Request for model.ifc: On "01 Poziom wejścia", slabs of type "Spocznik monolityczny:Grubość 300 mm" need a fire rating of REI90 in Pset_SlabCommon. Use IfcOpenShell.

First a look at what the model holds.

```python
import ifcopenshell
import ifcopenshell.util.element

model = ifcopenshell.open("model.ifc")
print(model.schema)
storey = next(s for s in model.by_type("IfcBuildingStorey") if s.Name == "01 Poziom wejścia")
slabs = [e for e in ifcopenshell.util.element.get_decomposition(storey) if e.is_a("IfcSlab")]
seen = {}
for e in slabs:
    element_type = ifcopenshell.util.element.get_type(e)
    key = (element_type.Name if element_type != e and element_type else None, ifcopenshell.util.element.get_pset(e, "Pset_SlabCommon", "FireRating"))
    seen[key] = seen.get(key, 0) + 1
for (name, value), count in sorted(seen.items(), key=str):
    print(count, "x", name, "|", value)
```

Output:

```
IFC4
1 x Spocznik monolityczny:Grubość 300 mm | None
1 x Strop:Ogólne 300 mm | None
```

```python
import ifcopenshell
import ifcopenshell.api.pset
import ifcopenshell.util.element

model = ifcopenshell.open("model.ifc")

storey = next(s for s in model.by_type("IfcBuildingStorey") if s.Name == "01 Poziom wejścia")
slabs = [e for e in ifcopenshell.util.element.get_decomposition(storey) if e.is_a("IfcSlab")]

count = 0
for e in slabs:
    element_type = ifcopenshell.util.element.get_type(e)
    if element_type in (None, e) or element_type.Name != "Spocznik monolityczny:Grubość 300 mm":
        continue
    # add_pset returns the element's existing set when there is one.
    pset = ifcopenshell.api.pset.add_pset(model, product=e, name="Pset_SlabCommon")
    ifcopenshell.api.pset.edit_pset(model, pset=pset, properties={"FireRating": "REI90"})
    count += 1

print(count, "slabs updated")

model.write("model_updated.ifc")
```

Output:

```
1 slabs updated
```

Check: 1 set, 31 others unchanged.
